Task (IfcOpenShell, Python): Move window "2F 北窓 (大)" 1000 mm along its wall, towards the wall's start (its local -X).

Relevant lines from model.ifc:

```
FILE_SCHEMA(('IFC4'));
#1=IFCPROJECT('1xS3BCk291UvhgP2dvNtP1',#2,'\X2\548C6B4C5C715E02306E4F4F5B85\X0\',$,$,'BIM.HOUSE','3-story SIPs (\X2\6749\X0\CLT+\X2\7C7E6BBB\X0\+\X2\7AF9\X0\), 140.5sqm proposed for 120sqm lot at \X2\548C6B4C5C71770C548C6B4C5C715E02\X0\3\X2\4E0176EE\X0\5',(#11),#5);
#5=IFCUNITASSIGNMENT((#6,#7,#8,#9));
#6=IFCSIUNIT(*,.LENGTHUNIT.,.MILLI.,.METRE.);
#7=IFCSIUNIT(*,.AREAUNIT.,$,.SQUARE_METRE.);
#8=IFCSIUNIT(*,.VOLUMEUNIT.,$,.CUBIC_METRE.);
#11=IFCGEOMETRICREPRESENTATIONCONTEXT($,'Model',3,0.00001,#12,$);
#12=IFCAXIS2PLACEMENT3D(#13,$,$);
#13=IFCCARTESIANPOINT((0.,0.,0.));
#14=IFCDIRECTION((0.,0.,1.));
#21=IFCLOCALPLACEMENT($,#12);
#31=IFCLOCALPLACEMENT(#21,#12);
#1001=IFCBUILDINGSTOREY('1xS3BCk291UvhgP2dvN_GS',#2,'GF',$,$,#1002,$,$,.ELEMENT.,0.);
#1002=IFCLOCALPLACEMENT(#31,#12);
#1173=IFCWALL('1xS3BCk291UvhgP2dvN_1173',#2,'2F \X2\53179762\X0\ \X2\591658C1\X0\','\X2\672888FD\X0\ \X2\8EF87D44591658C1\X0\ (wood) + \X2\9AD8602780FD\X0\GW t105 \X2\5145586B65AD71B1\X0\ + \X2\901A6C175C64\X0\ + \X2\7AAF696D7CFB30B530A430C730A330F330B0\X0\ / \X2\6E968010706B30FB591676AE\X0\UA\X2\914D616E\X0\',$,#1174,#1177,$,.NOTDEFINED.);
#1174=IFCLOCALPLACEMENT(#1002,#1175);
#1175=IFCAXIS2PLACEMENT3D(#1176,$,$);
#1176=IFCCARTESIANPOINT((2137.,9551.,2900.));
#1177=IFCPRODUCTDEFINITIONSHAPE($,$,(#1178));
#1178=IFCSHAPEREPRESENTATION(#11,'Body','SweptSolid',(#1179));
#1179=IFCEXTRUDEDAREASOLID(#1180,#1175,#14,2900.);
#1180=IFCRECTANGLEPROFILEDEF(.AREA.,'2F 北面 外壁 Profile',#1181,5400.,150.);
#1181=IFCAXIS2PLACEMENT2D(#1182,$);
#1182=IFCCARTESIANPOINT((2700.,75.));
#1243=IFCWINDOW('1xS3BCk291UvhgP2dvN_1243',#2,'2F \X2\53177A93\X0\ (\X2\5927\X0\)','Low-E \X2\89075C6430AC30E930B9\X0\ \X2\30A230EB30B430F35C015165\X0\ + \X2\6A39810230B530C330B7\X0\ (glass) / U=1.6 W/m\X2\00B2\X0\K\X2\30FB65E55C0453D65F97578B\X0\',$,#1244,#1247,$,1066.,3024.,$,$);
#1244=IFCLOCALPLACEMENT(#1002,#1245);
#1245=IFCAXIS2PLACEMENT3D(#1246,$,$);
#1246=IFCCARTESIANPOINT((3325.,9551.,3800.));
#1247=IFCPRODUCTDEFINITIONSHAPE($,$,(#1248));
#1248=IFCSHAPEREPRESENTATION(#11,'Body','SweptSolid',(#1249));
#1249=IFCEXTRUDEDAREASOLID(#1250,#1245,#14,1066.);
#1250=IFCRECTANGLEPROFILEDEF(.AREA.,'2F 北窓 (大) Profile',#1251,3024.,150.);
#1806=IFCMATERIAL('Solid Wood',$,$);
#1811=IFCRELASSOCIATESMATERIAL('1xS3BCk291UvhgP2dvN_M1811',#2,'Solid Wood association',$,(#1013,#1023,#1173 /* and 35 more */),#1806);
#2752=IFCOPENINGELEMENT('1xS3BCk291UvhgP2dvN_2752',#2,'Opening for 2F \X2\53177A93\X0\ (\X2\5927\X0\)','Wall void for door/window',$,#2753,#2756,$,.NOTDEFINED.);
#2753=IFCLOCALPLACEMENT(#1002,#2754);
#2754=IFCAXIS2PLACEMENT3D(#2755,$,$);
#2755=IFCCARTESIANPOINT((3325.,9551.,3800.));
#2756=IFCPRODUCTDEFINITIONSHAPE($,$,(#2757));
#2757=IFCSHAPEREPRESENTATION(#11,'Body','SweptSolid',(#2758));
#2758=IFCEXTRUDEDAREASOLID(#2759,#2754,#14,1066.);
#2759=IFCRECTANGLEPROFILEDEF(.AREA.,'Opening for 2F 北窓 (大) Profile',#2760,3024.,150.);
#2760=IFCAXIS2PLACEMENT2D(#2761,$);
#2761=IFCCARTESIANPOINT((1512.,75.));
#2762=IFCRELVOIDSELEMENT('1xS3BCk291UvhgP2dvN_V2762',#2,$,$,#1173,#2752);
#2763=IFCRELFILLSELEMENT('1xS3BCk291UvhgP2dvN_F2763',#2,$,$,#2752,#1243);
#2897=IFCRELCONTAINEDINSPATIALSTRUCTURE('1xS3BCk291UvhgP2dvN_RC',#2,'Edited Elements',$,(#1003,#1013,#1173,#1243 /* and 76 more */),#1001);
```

```python
import ifcopenshell
import ifcopenshell.api.geometry
import ifcopenshell.util.placement

model = ifcopenshell.open("model.ifc")

window = model.by_id(1243)
opening = window.FillsVoids[0].RelatingOpeningElement
wall = opening.VoidsElements[0].RelatingBuildingElement

wall_matrix = ifcopenshell.util.placement.get_local_placement(wall.ObjectPlacement)
shift = wall_matrix[:3, 0] * -1000.0
before = ifcopenshell.util.placement.get_local_placement(window.ObjectPlacement)[:3, 3].copy()

# The window is not placed relative to its opening, so move both.
for product in (opening, window):
    matrix = ifcopenshell.util.placement.get_local_placement(product.ObjectPlacement)
    matrix[:3, 3] += shift
    ifcopenshell.api.geometry.edit_object_placement(model, product=product, matrix=matrix, is_si=False)

after = ifcopenshell.util.placement.get_local_placement(window.ObjectPlacement)[:3, 3]
print("window moved by", (after - before).round(3) + 0.0)

model.write("model_edited.ifc")
```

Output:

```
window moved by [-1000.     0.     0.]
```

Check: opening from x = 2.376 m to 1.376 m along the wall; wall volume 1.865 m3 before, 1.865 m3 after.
